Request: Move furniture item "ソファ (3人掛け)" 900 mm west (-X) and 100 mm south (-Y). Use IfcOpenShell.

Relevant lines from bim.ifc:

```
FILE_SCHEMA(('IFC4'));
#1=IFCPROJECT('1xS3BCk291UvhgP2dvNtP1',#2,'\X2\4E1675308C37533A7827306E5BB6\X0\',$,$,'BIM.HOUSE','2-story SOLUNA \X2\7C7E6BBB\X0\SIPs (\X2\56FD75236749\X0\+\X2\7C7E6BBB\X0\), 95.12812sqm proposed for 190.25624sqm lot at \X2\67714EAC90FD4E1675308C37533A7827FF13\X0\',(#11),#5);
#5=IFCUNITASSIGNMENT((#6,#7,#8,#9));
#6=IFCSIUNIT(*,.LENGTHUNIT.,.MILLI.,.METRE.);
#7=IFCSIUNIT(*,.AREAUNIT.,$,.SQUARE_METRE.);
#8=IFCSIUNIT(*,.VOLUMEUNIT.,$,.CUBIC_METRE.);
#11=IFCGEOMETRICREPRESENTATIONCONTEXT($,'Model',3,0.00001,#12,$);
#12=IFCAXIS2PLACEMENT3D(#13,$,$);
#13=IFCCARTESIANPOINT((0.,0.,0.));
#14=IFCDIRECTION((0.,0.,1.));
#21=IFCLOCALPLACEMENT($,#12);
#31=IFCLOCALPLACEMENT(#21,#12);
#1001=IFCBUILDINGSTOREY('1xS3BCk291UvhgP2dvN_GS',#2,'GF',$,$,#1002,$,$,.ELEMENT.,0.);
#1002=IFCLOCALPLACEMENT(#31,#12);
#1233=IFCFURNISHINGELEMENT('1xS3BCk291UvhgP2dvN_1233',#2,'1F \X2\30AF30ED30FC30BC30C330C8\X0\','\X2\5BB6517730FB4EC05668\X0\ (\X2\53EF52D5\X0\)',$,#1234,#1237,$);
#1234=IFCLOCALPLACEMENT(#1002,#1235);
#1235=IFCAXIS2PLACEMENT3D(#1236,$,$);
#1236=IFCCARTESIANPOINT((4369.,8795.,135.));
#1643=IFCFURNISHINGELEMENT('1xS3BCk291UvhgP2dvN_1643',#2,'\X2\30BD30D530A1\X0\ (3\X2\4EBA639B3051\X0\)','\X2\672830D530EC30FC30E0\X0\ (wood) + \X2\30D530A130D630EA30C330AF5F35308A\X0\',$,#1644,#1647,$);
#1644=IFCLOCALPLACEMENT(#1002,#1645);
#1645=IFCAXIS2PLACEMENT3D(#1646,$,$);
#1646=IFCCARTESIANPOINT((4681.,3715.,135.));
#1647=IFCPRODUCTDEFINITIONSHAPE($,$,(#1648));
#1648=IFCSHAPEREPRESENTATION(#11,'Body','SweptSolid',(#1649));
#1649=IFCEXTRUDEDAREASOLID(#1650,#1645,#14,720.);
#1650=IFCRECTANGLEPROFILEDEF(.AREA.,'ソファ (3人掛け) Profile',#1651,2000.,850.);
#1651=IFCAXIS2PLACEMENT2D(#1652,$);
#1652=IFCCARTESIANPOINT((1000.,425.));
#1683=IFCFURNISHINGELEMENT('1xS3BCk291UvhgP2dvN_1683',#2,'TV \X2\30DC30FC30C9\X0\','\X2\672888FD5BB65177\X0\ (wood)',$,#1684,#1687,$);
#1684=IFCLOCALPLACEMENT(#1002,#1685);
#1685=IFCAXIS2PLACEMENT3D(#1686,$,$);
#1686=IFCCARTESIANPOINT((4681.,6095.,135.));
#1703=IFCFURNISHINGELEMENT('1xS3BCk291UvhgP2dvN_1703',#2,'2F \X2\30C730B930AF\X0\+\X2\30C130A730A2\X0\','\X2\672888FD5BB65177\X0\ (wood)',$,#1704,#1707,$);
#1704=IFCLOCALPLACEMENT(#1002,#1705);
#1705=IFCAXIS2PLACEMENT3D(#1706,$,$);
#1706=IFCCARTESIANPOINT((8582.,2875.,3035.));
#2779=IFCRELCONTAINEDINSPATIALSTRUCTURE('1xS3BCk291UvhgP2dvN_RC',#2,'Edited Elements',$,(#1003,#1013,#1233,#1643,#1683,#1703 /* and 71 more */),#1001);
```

```python
import ifcopenshell
import ifcopenshell.api.geometry
import ifcopenshell.util.placement
import ifcopenshell.util.unit

model = ifcopenshell.open("bim.ifc")
unit_scale = ifcopenshell.util.unit.calculate_unit_scale(model)

item = model.by_guid("1xS3BCk291UvhgP2dvN_1643")
matrix = ifcopenshell.util.placement.get_local_placement(item.ObjectPlacement)
matrix[0, 3] -= 0.9 / unit_scale
matrix[1, 3] -= 0.1 / unit_scale
ifcopenshell.api.geometry.edit_object_placement(model, product=item, matrix=matrix, is_si=False)

print(ifcopenshell.util.placement.get_local_placement(item.ObjectPlacement).round(3) + 0.0)

model.write("bim_v2.ifc")
```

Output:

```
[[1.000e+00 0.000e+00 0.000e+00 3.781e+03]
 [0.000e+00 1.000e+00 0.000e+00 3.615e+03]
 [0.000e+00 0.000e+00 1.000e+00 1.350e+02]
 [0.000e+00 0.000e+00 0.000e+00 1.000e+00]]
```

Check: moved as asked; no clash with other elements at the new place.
